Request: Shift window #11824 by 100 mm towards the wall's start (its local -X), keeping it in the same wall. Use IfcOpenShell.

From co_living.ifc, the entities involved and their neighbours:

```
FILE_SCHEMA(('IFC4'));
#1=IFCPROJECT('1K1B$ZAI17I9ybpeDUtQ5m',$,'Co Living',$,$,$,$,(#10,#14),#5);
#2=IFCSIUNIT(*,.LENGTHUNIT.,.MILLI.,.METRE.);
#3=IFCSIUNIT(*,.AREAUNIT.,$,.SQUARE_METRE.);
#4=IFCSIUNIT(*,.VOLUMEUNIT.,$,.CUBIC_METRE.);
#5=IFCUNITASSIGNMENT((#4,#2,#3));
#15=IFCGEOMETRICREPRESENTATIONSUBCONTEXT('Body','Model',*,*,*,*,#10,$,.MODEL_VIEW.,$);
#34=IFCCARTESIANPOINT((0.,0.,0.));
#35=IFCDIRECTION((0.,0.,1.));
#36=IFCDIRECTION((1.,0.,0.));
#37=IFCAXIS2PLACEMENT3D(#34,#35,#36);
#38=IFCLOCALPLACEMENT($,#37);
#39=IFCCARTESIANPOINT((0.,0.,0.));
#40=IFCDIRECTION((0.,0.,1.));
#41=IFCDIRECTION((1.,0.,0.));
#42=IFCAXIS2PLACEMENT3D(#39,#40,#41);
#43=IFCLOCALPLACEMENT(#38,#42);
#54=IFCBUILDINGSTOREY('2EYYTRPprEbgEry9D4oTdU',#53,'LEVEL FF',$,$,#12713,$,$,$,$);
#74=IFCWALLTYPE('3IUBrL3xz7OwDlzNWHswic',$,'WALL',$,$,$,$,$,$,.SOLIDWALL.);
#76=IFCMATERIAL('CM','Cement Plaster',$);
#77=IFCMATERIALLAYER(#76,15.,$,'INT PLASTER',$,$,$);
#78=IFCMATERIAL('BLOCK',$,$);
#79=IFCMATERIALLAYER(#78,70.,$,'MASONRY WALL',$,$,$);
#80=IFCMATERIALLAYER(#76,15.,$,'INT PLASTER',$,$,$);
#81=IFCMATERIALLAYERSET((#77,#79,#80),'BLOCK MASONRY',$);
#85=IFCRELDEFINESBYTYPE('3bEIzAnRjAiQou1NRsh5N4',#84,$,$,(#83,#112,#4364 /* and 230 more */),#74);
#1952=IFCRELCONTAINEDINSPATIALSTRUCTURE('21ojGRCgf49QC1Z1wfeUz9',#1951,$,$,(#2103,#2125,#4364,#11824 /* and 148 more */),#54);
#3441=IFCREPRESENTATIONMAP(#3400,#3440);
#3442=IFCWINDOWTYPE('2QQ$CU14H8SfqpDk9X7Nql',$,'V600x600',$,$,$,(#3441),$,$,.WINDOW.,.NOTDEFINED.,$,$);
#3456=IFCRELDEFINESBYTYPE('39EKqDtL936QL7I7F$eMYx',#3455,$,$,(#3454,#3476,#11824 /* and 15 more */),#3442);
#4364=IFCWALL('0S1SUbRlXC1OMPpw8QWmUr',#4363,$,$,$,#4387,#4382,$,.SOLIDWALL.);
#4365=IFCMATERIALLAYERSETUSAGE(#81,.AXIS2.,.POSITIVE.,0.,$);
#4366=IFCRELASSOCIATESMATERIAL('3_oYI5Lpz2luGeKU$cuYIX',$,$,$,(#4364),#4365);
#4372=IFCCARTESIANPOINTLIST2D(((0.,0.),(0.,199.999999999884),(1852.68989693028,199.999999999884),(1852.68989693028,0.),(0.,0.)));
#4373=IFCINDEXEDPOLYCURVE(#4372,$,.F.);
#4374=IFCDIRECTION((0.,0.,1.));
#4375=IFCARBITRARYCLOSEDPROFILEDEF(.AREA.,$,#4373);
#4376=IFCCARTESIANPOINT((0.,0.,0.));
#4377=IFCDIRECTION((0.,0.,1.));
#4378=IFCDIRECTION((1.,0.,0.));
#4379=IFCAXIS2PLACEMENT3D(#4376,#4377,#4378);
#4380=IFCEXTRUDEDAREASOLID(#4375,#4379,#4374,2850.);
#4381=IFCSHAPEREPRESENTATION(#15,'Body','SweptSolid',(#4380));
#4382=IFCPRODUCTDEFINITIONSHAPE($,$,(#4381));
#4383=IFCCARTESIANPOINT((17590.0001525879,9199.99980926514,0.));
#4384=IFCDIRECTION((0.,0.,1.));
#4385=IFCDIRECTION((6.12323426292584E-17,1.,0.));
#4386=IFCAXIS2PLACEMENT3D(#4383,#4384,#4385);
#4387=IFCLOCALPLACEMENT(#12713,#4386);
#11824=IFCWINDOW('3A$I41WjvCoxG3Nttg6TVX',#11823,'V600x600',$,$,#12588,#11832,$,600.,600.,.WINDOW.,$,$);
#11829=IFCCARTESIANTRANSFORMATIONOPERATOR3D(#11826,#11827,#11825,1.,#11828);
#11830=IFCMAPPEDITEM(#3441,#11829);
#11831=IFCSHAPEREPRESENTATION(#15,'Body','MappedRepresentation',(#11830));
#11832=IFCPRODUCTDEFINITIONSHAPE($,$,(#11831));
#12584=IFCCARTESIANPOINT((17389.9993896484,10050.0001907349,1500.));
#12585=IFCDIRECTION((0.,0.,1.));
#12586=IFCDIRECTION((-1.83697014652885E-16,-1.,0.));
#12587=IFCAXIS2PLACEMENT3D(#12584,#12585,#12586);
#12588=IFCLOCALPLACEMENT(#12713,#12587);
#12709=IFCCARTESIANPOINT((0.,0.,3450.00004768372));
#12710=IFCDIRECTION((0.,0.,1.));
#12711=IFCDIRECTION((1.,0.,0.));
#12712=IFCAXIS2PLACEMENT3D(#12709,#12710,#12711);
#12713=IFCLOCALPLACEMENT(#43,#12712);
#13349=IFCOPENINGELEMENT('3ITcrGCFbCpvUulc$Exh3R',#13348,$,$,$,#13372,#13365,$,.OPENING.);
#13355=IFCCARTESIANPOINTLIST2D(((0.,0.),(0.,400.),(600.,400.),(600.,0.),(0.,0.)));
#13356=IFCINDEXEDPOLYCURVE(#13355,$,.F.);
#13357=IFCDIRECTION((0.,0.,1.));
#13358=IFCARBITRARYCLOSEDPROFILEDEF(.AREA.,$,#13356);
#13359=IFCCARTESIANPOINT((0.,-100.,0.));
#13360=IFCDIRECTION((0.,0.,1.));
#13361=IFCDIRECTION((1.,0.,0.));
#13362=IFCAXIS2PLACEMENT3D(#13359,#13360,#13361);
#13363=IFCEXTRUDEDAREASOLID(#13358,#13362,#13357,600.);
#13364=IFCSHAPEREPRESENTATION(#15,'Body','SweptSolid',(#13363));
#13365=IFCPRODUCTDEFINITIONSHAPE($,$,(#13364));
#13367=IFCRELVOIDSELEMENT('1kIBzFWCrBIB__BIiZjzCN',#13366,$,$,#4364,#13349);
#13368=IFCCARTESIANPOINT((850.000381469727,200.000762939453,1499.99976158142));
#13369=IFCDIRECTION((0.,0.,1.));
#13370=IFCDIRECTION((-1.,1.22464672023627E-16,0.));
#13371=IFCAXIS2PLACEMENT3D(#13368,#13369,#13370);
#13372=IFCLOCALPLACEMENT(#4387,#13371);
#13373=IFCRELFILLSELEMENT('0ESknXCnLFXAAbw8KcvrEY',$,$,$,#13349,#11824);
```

```python
import ifcopenshell
import ifcopenshell.api.geometry
import ifcopenshell.util.placement
import ifcopenshell.util.unit

model = ifcopenshell.open("co_living.ifc")
unit_scale = ifcopenshell.util.unit.calculate_unit_scale(model)

window = model.by_guid("3A$I41WjvCoxG3Nttg6TVX")
opening = window.FillsVoids[0].RelatingOpeningElement
wall = opening.VoidsElements[0].RelatingBuildingElement

wall_matrix = ifcopenshell.util.placement.get_local_placement(wall.ObjectPlacement)
shift = wall_matrix[:3, 0] * -0.1 / unit_scale
before = ifcopenshell.util.placement.get_local_placement(window.ObjectPlacement)[:3, 3].copy()

# The window is not placed relative to its opening, so move both.
for product in (opening, window):
    matrix = ifcopenshell.util.placement.get_local_placement(product.ObjectPlacement)
    matrix[:3, 3] += shift
    ifcopenshell.api.geometry.edit_object_placement(model, product=product, matrix=matrix, is_si=False)

after = ifcopenshell.util.placement.get_local_placement(window.ObjectPlacement)[:3, 3]
print("window moved by", (after - before).round(3) + 0.0)

model.write("co_living-out.ifc")
```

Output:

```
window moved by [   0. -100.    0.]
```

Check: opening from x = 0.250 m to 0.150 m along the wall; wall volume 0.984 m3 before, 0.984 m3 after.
